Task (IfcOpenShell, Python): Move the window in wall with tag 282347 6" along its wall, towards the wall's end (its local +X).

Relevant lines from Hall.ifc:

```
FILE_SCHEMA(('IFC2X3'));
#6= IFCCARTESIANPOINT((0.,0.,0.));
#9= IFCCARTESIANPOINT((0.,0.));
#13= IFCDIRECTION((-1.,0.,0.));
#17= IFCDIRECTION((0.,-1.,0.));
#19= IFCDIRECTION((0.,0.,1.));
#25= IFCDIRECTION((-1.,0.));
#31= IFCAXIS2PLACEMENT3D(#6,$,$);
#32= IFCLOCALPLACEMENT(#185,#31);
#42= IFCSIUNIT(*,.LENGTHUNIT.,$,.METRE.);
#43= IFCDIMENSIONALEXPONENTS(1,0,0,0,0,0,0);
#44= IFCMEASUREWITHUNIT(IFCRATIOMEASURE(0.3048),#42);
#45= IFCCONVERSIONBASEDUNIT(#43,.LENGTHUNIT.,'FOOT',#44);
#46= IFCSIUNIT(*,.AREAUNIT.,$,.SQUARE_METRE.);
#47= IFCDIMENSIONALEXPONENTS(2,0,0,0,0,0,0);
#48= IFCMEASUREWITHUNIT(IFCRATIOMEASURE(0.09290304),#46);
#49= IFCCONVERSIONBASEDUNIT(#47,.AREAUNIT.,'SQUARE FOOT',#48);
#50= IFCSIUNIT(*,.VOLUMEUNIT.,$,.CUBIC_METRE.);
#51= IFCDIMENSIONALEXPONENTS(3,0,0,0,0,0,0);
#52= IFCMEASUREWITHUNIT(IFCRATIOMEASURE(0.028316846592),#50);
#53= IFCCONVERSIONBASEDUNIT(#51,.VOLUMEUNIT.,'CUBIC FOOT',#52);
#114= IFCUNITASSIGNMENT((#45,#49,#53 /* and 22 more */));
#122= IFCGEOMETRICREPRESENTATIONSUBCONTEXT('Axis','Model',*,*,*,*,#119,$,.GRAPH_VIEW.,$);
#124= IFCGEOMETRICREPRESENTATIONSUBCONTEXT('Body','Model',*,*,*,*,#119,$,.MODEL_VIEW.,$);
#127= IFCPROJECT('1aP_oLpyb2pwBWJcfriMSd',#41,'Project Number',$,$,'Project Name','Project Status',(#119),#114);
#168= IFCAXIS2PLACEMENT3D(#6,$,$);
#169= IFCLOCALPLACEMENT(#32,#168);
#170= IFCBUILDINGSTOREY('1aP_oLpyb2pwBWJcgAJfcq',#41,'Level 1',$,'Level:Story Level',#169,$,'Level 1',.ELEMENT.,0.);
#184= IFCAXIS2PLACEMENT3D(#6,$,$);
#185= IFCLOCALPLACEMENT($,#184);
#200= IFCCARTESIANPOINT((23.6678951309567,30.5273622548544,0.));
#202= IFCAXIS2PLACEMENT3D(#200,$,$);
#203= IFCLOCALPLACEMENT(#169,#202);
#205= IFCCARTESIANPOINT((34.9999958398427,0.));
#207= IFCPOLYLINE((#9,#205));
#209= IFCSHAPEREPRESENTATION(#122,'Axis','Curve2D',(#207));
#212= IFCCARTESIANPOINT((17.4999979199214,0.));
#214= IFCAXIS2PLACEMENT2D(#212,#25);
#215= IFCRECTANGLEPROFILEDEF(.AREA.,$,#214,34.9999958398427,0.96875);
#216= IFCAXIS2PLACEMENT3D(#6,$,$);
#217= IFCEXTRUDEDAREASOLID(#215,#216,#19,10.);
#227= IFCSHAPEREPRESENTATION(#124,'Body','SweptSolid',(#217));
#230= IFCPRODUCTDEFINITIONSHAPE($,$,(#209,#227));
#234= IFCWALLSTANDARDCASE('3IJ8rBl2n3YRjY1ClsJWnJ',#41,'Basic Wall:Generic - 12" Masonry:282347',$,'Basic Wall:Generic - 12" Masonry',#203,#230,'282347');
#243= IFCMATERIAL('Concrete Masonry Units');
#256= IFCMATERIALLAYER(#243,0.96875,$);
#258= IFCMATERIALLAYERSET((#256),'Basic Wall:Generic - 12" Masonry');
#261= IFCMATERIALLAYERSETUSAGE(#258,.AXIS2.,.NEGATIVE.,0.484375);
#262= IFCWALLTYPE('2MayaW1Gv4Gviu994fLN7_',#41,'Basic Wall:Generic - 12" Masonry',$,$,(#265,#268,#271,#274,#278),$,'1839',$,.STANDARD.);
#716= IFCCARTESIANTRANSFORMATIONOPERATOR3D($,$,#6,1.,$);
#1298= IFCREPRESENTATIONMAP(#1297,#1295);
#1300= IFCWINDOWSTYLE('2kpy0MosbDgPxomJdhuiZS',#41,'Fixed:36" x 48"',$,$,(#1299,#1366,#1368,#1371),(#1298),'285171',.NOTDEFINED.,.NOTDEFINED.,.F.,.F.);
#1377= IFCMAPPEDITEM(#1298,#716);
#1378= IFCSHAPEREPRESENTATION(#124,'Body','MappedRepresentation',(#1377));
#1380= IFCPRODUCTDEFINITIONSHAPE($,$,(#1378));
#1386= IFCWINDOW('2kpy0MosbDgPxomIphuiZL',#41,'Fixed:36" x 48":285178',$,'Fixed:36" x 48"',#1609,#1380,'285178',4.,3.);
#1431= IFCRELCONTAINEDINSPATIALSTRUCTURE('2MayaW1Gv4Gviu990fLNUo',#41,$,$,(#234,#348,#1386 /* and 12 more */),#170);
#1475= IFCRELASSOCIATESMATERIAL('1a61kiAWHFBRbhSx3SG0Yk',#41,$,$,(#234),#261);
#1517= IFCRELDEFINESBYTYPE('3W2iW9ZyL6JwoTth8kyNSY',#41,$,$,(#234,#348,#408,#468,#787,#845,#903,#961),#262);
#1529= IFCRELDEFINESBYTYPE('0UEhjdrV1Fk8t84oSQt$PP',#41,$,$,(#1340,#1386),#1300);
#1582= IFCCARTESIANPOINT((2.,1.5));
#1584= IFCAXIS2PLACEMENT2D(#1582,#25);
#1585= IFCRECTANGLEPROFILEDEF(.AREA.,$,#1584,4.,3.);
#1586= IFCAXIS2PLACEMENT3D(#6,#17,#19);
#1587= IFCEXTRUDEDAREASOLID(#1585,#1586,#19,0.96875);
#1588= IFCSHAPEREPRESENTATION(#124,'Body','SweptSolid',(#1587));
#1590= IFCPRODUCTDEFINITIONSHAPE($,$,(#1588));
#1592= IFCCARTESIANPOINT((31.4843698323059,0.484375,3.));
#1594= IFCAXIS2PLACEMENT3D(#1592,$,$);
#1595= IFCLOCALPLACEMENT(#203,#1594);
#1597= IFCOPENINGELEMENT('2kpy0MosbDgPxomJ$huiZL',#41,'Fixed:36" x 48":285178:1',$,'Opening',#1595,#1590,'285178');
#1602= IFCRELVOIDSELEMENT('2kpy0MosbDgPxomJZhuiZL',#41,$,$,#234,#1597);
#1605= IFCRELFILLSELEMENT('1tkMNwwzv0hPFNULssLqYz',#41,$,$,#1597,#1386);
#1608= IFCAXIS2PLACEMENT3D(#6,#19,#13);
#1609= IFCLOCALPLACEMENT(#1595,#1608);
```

```python
import ifcopenshell
import ifcopenshell.api.geometry
import ifcopenshell.util.placement
import ifcopenshell.util.unit

model = ifcopenshell.open("Hall.ifc")
unit_scale = ifcopenshell.util.unit.calculate_unit_scale(model)

window = model.by_id(1386)
opening = window.FillsVoids[0].RelatingOpeningElement
wall = opening.VoidsElements[0].RelatingBuildingElement

wall_matrix = ifcopenshell.util.placement.get_local_placement(wall.ObjectPlacement)
shift = wall_matrix[:3, 0] * 6 * 0.0254 / unit_scale
before = ifcopenshell.util.placement.get_local_placement(window.ObjectPlacement)[:3, 3].copy()

# The window is placed relative to its opening, so it follows when the opening moves.
matrix = ifcopenshell.util.placement.get_local_placement(opening.ObjectPlacement)
matrix[:3, 3] += shift
ifcopenshell.api.geometry.edit_object_placement(
    model, product=opening, matrix=matrix, is_si=False, should_transform_children=True
)

after = ifcopenshell.util.placement.get_local_placement(window.ObjectPlacement)[:3, 3]
print("window moved by", (after - before).round(3) + 0.0)

model.write("Hall_v2.ifc")
```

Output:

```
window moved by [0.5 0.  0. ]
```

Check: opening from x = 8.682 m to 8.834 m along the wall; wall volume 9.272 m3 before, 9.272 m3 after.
